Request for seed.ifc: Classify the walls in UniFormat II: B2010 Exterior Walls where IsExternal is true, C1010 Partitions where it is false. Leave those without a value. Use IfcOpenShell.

First a look at what the model holds.

```python
import ifcopenshell
import ifcopenshell.util.element

model = ifcopenshell.open("seed.ifc")
print(model.schema)
print("classifications:", [c.Name for c in model.by_type("IfcClassification")])
values = [ifcopenshell.util.element.get_pset(e, "Pset_WallCommon", "IsExternal") for e in model.by_type("IfcWall")]
for value in (True, False, None):
    print("IsExternal", value, values.count(value))
```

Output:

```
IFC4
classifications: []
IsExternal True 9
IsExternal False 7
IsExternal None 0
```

```python
import ifcopenshell
import ifcopenshell.api.classification
import ifcopenshell.util.element

model = ifcopenshell.open("seed.ifc")

system = ifcopenshell.api.classification.add_classification(model, classification="UniFormat II")

walls = model.by_type("IfcWall")
external = {e: ifcopenshell.util.element.get_pset(e, "Pset_WallCommon", "IsExternal") for e in walls}
for flag, code, name in ((True, "B2010", "Exterior Walls"), (False, "C1010", "Partitions")):
    products = [e for e in walls if external[e] is flag]
    ifcopenshell.api.classification.add_reference(
        model, products=products, classification=system, identification=code, name=name
    )
    print(code, len(products))

model.write("seed_edited.ifc")
```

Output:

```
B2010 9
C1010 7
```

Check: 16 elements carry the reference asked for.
